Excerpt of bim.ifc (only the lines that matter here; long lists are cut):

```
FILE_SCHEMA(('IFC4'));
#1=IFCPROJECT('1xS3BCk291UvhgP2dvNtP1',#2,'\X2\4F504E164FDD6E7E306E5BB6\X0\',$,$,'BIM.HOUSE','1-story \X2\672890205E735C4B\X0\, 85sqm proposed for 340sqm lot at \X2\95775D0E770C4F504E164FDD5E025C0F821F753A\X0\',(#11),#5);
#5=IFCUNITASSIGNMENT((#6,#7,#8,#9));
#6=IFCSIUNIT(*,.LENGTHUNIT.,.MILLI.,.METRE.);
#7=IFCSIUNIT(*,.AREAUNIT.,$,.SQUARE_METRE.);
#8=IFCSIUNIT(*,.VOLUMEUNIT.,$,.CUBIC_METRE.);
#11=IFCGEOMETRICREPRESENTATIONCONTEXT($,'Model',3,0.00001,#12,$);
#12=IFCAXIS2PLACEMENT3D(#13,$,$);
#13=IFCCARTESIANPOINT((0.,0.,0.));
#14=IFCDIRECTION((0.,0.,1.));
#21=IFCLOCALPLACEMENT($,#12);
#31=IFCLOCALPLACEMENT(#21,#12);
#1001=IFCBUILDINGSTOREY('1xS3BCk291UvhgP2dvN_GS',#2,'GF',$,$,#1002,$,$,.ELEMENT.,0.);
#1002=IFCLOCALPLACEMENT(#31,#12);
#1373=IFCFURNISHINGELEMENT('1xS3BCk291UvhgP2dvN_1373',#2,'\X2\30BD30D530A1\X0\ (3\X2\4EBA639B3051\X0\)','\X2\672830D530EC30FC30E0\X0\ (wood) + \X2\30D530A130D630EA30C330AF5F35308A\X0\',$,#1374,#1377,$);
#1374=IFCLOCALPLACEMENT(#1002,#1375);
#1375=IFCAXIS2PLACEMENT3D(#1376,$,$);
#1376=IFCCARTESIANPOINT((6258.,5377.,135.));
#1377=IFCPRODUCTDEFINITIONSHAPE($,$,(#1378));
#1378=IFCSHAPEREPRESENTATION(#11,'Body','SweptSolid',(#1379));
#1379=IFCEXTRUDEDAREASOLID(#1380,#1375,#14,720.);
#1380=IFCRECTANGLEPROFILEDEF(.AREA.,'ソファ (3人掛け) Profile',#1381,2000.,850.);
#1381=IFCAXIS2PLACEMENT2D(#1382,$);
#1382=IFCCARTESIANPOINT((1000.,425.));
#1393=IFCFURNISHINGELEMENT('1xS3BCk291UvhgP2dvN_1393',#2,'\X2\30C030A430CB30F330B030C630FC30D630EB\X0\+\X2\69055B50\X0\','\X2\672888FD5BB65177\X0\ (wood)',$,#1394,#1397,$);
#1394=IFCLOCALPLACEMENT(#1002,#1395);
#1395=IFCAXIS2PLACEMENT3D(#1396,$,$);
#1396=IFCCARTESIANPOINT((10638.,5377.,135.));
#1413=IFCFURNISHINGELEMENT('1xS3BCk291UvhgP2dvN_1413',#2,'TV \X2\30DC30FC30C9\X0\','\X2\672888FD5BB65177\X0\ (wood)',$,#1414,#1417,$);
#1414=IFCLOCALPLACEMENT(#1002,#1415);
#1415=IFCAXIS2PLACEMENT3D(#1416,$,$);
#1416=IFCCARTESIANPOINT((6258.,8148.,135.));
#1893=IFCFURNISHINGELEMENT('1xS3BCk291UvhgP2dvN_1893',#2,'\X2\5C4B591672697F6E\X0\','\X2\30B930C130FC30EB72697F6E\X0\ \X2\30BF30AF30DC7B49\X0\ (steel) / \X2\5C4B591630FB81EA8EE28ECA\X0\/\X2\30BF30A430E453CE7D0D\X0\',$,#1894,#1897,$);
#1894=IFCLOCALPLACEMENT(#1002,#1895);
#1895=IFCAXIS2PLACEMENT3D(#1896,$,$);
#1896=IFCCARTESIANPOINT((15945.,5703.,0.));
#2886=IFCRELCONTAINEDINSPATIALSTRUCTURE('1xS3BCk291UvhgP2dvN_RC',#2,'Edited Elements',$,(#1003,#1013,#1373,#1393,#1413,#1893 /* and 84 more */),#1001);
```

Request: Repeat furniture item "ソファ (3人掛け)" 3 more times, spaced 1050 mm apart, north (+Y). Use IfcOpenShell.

```python
import numpy as np
import ifcopenshell
import ifcopenshell.api.geometry
import ifcopenshell.api.root
import ifcopenshell.util.element
import ifcopenshell.util.placement
import ifcopenshell.util.unit

model = ifcopenshell.open("bim.ifc")
unit_scale = ifcopenshell.util.unit.calculate_unit_scale(model)


def reuse_history(source, copy):
    """copy_class also copies each property set's owner history, people and application; keep the originals."""
    for rel in copy.IsDefinedBy:
        if rel.is_a("IfcRelDefinesByProperties") and (history := rel.RelatingPropertyDefinition.OwnerHistory):
            rel.RelatingPropertyDefinition.OwnerHistory = source.OwnerHistory
            ifcopenshell.util.element.remove_deep2(model, history)


source = model.by_id(1373)
base = ifcopenshell.util.placement.get_local_placement(source.ObjectPlacement)
step = np.array([0.0, 1.0, 0.0]) * 1.05 / unit_scale

for i in range(1, 4):
    copy = ifcopenshell.api.root.copy_class(model, product=source)
    copy.Representation = ifcopenshell.util.element.copy_deep(
        model, source.Representation, exclude=["IfcGeometricRepresentationContext", "IfcRepresentationMap"]
    )
    reuse_history(source, copy)
    matrix = base.copy()
    matrix[:3, 3] += i * step
    print("added at", matrix[:3, 3].round(3) + 0.0)
    ifcopenshell.api.geometry.edit_object_placement(model, product=copy, matrix=matrix, is_si=False)

model.write("bim-out.ifc")
```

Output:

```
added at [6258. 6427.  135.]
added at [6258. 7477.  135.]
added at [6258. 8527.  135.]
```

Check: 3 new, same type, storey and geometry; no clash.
